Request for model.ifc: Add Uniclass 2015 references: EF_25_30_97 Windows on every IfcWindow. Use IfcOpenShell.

First a look at what the model holds.

```python
import ifcopenshell

model = ifcopenshell.open("model.ifc")
print(model.schema)
print("classifications:", [c.Name for c in model.by_type("IfcClassification")])
for ifc_class in ("IfcDoor", "IfcRoof", "IfcStair", "IfcWall", "IfcWindow"):
    print(ifc_class, len(model.by_type(ifc_class)))
```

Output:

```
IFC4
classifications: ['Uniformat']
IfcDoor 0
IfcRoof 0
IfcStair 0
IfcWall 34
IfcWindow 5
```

```python
import ifcopenshell
import ifcopenshell.api.classification

model = ifcopenshell.open("model.ifc")

system = ifcopenshell.api.classification.add_classification(model, classification="Uniclass 2015")

codes = {
    "IfcWindow": ("EF_25_30_97", "Windows"),
}
for ifc_class, (code, name) in codes.items():
    products = model.by_type(ifc_class)
    ifcopenshell.api.classification.add_reference(
        model, products=products, classification=system, identification=code, name=name
    )
    print(code, len(products))

model.write("model-out.ifc")
```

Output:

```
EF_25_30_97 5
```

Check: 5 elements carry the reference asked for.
